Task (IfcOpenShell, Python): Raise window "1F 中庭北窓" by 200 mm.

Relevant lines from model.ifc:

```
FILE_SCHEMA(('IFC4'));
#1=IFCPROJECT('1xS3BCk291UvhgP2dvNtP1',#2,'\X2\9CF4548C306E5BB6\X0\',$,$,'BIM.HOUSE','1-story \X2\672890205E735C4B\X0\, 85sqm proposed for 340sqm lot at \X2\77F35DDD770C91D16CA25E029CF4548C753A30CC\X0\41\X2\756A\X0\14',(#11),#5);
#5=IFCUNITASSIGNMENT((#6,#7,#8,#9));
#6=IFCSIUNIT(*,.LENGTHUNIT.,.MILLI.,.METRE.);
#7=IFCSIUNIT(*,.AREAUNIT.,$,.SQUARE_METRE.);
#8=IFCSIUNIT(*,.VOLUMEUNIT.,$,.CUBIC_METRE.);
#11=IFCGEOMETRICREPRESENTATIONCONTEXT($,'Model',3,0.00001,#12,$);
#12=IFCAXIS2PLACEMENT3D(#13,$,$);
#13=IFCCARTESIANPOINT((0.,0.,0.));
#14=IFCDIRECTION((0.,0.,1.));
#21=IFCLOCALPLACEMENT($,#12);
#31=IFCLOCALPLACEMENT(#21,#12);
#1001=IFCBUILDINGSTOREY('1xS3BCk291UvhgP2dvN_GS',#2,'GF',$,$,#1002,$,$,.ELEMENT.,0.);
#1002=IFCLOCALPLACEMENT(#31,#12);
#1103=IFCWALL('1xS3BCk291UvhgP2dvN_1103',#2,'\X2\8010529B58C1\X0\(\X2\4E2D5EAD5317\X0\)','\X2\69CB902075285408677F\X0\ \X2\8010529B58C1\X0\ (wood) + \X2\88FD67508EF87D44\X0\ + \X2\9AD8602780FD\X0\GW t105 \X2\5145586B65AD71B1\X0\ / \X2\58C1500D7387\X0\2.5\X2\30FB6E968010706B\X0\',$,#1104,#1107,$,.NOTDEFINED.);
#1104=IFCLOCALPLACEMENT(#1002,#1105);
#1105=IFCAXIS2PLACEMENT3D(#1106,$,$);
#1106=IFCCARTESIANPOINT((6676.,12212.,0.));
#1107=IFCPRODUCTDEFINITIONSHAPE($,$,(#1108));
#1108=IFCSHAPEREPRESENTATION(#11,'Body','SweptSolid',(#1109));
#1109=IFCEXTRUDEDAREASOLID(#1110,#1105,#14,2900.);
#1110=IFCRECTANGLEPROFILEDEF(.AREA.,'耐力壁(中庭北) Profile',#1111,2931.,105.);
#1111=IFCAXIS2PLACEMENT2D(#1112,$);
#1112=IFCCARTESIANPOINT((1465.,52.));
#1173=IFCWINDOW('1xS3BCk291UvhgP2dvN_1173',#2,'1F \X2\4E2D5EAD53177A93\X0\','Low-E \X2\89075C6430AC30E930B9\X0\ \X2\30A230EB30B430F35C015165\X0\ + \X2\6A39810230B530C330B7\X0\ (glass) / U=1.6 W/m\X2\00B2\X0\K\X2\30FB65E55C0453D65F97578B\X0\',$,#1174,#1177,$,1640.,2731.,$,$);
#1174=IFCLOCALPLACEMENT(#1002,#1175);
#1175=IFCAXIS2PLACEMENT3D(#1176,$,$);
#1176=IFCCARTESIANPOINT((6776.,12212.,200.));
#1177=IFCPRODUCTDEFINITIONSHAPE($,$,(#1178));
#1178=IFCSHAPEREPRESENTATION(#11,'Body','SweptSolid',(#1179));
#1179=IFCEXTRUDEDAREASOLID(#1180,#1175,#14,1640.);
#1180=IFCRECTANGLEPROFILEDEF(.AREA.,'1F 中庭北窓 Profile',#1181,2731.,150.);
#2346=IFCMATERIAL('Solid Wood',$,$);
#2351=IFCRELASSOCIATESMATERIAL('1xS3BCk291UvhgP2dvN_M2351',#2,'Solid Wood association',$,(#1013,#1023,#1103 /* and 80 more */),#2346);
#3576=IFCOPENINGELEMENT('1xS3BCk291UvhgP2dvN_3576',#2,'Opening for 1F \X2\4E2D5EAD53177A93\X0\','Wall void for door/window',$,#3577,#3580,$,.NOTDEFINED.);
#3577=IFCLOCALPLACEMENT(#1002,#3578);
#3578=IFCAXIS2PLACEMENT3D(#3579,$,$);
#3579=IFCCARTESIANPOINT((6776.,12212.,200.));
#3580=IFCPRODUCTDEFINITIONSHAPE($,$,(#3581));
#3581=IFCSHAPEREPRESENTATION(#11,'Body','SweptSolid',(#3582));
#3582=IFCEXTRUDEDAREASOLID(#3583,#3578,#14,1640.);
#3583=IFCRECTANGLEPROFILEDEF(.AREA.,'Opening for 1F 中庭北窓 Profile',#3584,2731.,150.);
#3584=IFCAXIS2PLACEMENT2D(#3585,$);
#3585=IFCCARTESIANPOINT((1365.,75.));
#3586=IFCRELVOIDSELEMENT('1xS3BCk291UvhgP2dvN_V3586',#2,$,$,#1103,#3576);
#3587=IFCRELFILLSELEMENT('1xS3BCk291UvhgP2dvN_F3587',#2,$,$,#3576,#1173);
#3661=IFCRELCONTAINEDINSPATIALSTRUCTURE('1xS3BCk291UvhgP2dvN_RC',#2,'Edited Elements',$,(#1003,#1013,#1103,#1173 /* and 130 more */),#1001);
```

```python
import numpy as np
import ifcopenshell
import ifcopenshell.api.geometry
import ifcopenshell.util.placement
import ifcopenshell.util.unit

model = ifcopenshell.open("model.ifc")
unit_scale = ifcopenshell.util.unit.calculate_unit_scale(model)

window = model.by_guid("1xS3BCk291UvhgP2dvN_1173")
opening = window.FillsVoids[0].RelatingOpeningElement
dz = 0.2 / unit_scale

shift = np.array([0.0, 0.0, dz])
# The window is not placed relative to its opening, so move both.
for product in (opening, window):
    matrix = ifcopenshell.util.placement.get_local_placement(product.ObjectPlacement)
    matrix[:3, 3] += shift
    ifcopenshell.api.geometry.edit_object_placement(model, product=product, matrix=matrix, is_si=False)

print(f"moved by {dz * unit_scale:+.3f} m")

model.write("model_v2.ifc")
```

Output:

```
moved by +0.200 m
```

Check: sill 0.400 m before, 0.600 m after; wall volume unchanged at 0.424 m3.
